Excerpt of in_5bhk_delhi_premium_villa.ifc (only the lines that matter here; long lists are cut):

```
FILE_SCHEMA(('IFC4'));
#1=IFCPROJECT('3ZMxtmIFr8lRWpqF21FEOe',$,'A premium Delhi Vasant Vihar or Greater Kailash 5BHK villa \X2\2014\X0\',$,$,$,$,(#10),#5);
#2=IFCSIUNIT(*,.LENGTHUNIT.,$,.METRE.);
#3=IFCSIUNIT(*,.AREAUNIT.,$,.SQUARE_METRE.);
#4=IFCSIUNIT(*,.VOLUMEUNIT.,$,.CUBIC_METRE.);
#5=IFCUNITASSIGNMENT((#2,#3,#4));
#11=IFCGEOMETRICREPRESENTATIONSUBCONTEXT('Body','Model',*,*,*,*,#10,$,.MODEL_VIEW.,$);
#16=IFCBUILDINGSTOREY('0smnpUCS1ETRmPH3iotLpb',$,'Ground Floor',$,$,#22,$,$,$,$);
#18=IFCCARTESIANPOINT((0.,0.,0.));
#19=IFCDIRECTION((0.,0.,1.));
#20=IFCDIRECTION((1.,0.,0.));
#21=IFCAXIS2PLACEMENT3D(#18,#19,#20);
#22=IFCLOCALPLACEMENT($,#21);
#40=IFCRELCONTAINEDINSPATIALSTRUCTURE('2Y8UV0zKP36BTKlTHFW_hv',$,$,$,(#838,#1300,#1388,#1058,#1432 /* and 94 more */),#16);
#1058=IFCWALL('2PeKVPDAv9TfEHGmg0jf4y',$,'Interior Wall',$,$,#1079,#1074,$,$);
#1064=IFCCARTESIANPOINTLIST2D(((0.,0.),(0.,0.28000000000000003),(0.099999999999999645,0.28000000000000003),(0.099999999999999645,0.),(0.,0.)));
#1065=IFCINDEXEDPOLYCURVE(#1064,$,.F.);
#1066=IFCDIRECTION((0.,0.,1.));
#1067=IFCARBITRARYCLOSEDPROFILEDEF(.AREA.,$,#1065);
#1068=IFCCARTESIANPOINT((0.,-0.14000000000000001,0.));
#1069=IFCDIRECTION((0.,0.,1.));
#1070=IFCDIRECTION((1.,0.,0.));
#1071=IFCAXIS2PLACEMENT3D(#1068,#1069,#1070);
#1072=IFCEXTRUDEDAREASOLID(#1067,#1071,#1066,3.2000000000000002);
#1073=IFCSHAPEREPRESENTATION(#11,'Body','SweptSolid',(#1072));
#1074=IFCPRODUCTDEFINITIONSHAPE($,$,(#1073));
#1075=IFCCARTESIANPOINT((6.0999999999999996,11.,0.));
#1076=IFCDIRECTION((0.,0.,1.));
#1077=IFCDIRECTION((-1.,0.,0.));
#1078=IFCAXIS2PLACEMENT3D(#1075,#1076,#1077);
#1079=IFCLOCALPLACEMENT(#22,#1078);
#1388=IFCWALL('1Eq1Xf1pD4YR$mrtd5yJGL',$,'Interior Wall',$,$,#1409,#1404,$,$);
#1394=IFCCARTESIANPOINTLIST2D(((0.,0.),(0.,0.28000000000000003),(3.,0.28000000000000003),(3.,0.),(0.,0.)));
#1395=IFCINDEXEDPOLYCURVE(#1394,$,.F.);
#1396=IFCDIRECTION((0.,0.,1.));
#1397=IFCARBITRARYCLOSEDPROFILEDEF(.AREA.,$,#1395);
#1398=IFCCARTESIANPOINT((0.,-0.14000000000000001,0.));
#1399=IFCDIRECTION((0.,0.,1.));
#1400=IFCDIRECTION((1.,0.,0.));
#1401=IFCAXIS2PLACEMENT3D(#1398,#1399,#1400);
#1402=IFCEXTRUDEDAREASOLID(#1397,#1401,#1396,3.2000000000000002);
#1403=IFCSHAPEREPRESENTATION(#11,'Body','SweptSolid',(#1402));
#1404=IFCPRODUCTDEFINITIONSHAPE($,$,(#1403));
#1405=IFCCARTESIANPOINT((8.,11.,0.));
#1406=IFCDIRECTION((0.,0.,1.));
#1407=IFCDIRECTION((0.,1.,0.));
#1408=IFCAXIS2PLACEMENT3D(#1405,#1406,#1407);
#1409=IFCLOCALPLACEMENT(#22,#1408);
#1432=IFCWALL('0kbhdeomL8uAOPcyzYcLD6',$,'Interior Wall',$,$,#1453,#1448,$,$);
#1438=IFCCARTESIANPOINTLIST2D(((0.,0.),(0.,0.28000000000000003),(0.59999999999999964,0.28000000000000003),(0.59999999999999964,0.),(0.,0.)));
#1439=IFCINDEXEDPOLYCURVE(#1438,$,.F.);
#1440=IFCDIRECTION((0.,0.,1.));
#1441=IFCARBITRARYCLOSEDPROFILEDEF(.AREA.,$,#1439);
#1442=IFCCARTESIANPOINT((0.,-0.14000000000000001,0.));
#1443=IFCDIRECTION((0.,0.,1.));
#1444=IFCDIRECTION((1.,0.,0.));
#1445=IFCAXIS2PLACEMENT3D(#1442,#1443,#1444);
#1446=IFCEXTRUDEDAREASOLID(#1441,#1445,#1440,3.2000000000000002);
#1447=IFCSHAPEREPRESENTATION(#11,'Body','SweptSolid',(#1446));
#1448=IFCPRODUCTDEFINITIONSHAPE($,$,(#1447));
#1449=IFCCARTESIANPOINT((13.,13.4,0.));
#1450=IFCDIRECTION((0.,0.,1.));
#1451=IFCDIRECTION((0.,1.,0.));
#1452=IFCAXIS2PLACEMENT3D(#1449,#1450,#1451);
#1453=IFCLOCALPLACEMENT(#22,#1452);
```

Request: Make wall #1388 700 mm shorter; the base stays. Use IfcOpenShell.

```python
import ifcopenshell
import ifcopenshell.geom
import ifcopenshell.util.representation
import ifcopenshell.util.shape

model = ifcopenshell.open("in_5bhk_delhi_premium_villa.ifc")
settings = ifcopenshell.geom.settings()


def volume(element):
    """Net volume in cubic metres, openings subtracted."""
    shape = ifcopenshell.geom.create_shape(settings, element)
    return ifcopenshell.util.shape.get_volume(shape.geometry)


wall = model.by_guid("1Eq1Xf1pD4YR$mrtd5yJGL")
before = volume(wall)

body = ifcopenshell.util.representation.get_representation(wall, "Model", "Body")
solid = body.Items[0]
old_height = solid.Depth
solid.Depth -= 0.7
after = volume(wall)

print(f"height {old_height:g} -> {solid.Depth:g}, volume {before:.3f} -> {after:.3f} m3")

model.write("in_5bhk_delhi_premium_villa_v2.ifc")
```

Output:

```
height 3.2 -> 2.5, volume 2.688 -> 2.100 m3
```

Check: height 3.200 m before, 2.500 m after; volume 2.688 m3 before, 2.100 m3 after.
